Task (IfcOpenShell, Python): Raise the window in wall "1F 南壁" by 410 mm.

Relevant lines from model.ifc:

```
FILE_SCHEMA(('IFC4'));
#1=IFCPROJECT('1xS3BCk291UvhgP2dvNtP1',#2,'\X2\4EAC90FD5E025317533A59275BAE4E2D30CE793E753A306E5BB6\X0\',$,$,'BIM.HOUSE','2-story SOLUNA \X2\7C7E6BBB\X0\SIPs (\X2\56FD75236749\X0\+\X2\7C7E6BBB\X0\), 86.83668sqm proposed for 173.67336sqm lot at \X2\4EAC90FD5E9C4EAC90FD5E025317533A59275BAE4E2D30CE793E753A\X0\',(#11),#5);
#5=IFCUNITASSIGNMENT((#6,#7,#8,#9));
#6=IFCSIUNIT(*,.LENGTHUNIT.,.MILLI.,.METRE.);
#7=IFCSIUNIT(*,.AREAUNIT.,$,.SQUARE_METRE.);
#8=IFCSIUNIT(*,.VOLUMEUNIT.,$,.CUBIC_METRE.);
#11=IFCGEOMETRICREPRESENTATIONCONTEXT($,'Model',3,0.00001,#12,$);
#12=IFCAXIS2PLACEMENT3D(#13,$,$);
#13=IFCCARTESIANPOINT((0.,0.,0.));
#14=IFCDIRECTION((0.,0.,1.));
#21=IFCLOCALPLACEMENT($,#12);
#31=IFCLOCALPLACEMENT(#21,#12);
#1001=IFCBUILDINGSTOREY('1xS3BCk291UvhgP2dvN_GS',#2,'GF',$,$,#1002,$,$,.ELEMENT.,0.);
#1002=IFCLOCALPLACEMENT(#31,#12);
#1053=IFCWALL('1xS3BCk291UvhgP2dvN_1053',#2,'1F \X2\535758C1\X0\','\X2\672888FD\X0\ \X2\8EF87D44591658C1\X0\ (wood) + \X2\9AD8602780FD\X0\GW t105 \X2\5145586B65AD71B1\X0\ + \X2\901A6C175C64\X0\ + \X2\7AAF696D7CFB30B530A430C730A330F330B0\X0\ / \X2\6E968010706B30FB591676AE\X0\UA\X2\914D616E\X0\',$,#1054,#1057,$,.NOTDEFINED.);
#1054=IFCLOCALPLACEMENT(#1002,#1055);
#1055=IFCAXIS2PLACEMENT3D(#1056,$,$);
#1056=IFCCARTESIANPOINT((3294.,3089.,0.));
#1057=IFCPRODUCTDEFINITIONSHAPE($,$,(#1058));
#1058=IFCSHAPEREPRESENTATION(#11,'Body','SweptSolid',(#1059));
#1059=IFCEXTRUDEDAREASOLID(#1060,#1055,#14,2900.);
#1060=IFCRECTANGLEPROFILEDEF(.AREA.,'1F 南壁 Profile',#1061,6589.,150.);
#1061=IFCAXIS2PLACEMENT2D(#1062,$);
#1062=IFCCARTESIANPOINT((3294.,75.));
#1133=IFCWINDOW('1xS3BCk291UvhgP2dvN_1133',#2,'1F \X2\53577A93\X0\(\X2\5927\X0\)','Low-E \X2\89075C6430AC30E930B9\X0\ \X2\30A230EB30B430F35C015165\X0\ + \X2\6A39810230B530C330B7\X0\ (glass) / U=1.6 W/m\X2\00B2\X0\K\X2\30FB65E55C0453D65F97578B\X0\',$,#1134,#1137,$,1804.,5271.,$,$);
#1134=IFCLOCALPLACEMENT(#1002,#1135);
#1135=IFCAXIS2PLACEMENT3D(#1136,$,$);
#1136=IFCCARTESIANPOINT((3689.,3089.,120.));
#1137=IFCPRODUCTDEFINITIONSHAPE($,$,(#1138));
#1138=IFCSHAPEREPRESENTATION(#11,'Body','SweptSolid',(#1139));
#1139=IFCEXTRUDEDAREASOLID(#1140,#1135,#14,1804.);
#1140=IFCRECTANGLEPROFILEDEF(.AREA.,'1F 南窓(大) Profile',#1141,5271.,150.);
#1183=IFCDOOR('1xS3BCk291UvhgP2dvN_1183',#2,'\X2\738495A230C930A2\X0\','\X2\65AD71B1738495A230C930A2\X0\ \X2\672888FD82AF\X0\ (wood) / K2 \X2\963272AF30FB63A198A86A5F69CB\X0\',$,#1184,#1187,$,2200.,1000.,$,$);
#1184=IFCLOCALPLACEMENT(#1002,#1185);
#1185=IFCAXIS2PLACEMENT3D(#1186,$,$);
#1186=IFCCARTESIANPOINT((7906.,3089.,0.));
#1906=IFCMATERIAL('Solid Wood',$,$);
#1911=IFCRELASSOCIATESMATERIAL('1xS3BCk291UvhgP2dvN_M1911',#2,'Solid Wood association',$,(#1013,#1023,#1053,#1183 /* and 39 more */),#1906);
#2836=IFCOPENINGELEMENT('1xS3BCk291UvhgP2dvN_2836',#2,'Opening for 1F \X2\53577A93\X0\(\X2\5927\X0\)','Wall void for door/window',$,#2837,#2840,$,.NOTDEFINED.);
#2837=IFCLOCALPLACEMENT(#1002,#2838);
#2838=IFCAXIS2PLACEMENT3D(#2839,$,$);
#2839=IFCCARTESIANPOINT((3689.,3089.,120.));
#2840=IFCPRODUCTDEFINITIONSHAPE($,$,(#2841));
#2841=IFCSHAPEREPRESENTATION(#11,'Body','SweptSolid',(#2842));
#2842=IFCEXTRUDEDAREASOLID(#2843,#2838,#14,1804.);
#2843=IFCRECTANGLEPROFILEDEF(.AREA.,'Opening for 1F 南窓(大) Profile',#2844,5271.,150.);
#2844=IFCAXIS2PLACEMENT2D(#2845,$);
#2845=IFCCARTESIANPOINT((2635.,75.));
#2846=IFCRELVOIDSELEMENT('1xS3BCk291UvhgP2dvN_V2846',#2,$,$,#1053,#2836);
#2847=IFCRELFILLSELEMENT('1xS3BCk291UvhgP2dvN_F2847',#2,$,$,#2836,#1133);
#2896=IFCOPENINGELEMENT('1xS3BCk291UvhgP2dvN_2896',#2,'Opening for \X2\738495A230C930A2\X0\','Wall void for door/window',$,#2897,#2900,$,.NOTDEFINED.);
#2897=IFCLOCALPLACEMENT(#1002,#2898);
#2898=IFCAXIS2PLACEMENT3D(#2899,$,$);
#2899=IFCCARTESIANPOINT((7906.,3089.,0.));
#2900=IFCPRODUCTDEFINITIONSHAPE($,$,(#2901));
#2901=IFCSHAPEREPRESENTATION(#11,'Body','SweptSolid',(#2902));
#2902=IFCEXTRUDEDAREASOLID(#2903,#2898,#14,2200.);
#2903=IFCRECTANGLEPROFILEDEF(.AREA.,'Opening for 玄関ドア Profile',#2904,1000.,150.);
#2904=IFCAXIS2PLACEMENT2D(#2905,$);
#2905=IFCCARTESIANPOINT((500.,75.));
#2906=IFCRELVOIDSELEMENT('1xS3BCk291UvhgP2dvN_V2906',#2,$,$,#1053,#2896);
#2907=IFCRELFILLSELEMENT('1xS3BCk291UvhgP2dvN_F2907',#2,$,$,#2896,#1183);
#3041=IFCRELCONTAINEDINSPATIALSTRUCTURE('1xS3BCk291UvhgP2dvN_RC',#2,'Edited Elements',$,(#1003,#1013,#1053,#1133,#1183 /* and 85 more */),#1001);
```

```python
import numpy as np
import ifcopenshell
import ifcopenshell.api.geometry
import ifcopenshell.util.placement
import ifcopenshell.util.unit

model = ifcopenshell.open("model.ifc")
unit_scale = ifcopenshell.util.unit.calculate_unit_scale(model)

window = model.by_id(1133)
opening = window.FillsVoids[0].RelatingOpeningElement
dz = 0.41 / unit_scale

shift = np.array([0.0, 0.0, dz])
# The window is not placed relative to its opening, so move both.
for product in (opening, window):
    matrix = ifcopenshell.util.placement.get_local_placement(product.ObjectPlacement)
    matrix[:3, 3] += shift
    ifcopenshell.api.geometry.edit_object_placement(model, product=product, matrix=matrix, is_si=False)

print(f"moved by {dz * unit_scale:+.3f} m")

model.write("model_edited.ifc")
```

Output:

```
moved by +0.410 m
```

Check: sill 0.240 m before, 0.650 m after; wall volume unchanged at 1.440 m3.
